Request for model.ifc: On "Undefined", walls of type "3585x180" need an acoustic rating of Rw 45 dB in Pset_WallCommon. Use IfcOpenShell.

First a look at what the model holds.

```python
import ifcopenshell
import ifcopenshell.util.element

model = ifcopenshell.open("model.ifc")
print(model.schema)
storey = next(s for s in model.by_type("IfcBuildingStorey") if s.Name == "Undefined")
walls = [e for e in ifcopenshell.util.element.get_decomposition(storey) if e.is_a("IfcWall")]
seen = {}
for e in walls:
    element_type = ifcopenshell.util.element.get_type(e)
    key = (element_type.Name if element_type != e and element_type else None, ifcopenshell.util.element.get_pset(e, "Pset_WallCommon", "AcousticRating"))
    seen[key] = seen.get(key, 0) + 1
for (name, value), count in sorted(seen.items(), key=str):
    print(count, "x", name, "|", value)
```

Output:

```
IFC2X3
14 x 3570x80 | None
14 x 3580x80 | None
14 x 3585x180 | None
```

```python
import ifcopenshell
import ifcopenshell.api.pset
import ifcopenshell.util.element

model = ifcopenshell.open("model.ifc")

storey = next(s for s in model.by_type("IfcBuildingStorey") if s.Name == "Undefined")
walls = [e for e in ifcopenshell.util.element.get_decomposition(storey) if e.is_a("IfcWall")]

count = 0
for e in walls:
    element_type = ifcopenshell.util.element.get_type(e)
    if element_type in (None, e) or element_type.Name != "3585x180":
        continue
    found = ifcopenshell.util.element.get_pset(e, "Pset_WallCommon", should_inherit=False)
    if found:
        pset = model.by_id(found["id"])
        if len(ifcopenshell.util.element.get_elements_by_pset(pset)) > 1:
            pset = ifcopenshell.api.pset.unshare_pset(model, products=[e], pset=pset)[0]
    else:
        pset = ifcopenshell.api.pset.add_pset(model, product=e, name="Pset_WallCommon")
    ifcopenshell.api.pset.edit_pset(model, pset=pset, properties={"AcousticRating": "Rw 45 dB"})
    count += 1

print(count, "walls updated")

model.write("model_edited.ifc")
```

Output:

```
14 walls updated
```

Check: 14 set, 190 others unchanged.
